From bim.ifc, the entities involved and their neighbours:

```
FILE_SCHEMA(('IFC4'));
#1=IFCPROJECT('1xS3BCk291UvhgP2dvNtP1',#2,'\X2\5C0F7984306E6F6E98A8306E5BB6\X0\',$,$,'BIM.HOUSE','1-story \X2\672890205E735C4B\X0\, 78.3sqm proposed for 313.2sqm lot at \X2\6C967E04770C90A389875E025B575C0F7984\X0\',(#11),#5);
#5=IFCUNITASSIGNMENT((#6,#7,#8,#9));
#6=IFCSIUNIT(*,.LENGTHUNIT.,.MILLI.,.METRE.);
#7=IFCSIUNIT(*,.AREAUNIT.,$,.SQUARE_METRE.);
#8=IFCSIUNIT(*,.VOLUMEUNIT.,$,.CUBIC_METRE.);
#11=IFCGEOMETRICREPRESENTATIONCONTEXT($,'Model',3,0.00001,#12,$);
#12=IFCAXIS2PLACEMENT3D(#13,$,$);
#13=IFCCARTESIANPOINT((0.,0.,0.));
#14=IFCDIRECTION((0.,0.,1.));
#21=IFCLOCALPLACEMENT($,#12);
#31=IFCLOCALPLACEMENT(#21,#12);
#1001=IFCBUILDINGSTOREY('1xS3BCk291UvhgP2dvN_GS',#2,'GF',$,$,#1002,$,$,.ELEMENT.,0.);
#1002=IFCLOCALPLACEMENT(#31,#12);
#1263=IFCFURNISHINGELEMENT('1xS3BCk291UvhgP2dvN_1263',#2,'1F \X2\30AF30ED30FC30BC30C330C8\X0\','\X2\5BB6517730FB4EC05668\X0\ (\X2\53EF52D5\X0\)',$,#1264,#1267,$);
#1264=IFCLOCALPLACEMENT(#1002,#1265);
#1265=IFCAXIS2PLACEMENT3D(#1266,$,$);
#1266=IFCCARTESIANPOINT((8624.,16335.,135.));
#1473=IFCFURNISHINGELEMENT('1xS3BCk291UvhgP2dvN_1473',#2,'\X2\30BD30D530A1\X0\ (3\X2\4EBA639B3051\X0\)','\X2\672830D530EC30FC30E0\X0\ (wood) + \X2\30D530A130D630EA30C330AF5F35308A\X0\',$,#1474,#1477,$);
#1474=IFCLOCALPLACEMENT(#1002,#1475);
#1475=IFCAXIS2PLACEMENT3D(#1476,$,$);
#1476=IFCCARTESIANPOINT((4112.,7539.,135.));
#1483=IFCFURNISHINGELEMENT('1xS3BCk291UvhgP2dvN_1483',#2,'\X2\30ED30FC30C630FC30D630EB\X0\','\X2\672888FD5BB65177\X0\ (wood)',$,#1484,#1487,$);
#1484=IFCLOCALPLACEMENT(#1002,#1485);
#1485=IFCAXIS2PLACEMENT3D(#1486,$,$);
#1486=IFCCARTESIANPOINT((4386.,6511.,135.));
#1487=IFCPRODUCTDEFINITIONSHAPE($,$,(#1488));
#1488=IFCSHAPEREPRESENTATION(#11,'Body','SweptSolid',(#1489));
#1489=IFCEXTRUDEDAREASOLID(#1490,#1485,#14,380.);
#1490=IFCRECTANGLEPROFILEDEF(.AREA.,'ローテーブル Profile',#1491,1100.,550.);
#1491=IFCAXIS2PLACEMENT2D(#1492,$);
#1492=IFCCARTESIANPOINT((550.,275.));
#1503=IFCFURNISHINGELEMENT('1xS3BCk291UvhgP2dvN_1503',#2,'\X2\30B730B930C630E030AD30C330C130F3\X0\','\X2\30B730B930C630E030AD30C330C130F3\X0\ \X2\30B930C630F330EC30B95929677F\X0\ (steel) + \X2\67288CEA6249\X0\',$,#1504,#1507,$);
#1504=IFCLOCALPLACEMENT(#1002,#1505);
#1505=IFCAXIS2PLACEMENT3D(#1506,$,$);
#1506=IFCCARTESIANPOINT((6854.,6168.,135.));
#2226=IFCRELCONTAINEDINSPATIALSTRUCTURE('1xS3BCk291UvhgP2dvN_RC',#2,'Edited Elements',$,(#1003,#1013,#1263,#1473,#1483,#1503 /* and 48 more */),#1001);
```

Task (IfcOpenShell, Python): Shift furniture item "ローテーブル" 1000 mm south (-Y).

```python
import ifcopenshell
import ifcopenshell.api.geometry
import ifcopenshell.util.placement
import ifcopenshell.util.unit

model = ifcopenshell.open("bim.ifc")
unit_scale = ifcopenshell.util.unit.calculate_unit_scale(model)

item = model.by_guid("1xS3BCk291UvhgP2dvN_1483")
matrix = ifcopenshell.util.placement.get_local_placement(item.ObjectPlacement)
matrix[1, 3] -= 1 / unit_scale
ifcopenshell.api.geometry.edit_object_placement(model, product=item, matrix=matrix, is_si=False)

print(ifcopenshell.util.placement.get_local_placement(item.ObjectPlacement).round(3) + 0.0)

model.write("bim_rev.ifc")
```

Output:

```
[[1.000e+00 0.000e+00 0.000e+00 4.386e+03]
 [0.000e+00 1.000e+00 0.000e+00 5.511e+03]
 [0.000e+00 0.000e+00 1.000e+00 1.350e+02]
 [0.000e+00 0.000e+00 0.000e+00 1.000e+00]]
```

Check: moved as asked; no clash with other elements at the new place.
